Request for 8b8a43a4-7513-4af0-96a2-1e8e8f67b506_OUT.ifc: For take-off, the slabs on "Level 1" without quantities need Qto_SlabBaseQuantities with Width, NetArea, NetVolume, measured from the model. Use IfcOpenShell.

First a look at what the model holds.

```python
import ifcopenshell
import ifcopenshell.util.element
import ifcopenshell.util.unit

model = ifcopenshell.open("8b8a43a4-7513-4af0-96a2-1e8e8f67b506_OUT.ifc")
print(model.schema)
for unit_type in ("LENGTHUNIT", "AREAUNIT", "VOLUMEUNIT"):
    print(unit_type, ifcopenshell.util.unit.calculate_unit_scale(model, unit_type))
storey = next(s for s in model.by_type("IfcBuildingStorey") if s.Name == "Level 1")
slabs = [e for e in ifcopenshell.util.element.get_decomposition(storey) if e.is_a("IfcSlab")]
for e in sorted(slabs, key=lambda e: e.id()):
    print(e.id(), e.is_a(), e.Name, list(ifcopenshell.util.element.get_psets(e, qtos_only=True)), sep=" | ")
```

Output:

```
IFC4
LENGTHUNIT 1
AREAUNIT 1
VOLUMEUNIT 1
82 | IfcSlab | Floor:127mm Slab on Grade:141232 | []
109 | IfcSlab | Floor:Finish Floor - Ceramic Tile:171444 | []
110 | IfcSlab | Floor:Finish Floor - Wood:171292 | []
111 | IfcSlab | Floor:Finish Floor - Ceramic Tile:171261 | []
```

```python
import ifcopenshell
import ifcopenshell.api.pset
import ifcopenshell.geom
import ifcopenshell.util.element
import ifcopenshell.util.shape
import ifcopenshell.util.unit

model = ifcopenshell.open("8b8a43a4-7513-4af0-96a2-1e8e8f67b506_OUT.ifc")
unit_scale = ifcopenshell.util.unit.calculate_unit_scale(model)
area_scale = ifcopenshell.util.unit.calculate_unit_scale(model, "AREAUNIT")
volume_scale = ifcopenshell.util.unit.calculate_unit_scale(model, "VOLUMEUNIT")
settings = ifcopenshell.geom.settings()

storey = next(s for s in model.by_type("IfcBuildingStorey") if s.Name == "Level 1")
slabs = [e for e in ifcopenshell.util.element.get_decomposition(storey) if e.is_a("IfcSlab")]

for e in sorted(slabs, key=lambda e: e.id()):
    if ifcopenshell.util.element.get_psets(e, qtos_only=True, should_inherit=False):
        continue
    # Geometry comes back in metres, in the element's own axes.
    shape = ifcopenshell.geom.create_shape(settings, e)
    values = {
        "Width": ifcopenshell.util.shape.get_z(shape.geometry) / unit_scale,
        "NetArea": ifcopenshell.util.shape.get_footprint_area(shape.geometry) / area_scale,
        "NetVolume": ifcopenshell.util.shape.get_volume(shape.geometry) / volume_scale,
    }
    qto = ifcopenshell.api.pset.add_qto(model, product=e, name="Qto_SlabBaseQuantities")
    ifcopenshell.api.pset.edit_qto(model, qto=qto, properties=values)
    print(e.id(), {k: round(v, 3) for k, v in values.items()})

model.write("8b8a43a4-7513-4af0-96a2-1e8e8f67b506_OUT_rev.ifc")
```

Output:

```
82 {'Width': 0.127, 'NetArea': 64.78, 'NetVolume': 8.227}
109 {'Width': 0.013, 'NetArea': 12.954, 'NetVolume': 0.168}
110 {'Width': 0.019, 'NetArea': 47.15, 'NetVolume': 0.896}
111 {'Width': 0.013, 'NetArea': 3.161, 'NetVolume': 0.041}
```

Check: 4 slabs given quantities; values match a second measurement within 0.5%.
